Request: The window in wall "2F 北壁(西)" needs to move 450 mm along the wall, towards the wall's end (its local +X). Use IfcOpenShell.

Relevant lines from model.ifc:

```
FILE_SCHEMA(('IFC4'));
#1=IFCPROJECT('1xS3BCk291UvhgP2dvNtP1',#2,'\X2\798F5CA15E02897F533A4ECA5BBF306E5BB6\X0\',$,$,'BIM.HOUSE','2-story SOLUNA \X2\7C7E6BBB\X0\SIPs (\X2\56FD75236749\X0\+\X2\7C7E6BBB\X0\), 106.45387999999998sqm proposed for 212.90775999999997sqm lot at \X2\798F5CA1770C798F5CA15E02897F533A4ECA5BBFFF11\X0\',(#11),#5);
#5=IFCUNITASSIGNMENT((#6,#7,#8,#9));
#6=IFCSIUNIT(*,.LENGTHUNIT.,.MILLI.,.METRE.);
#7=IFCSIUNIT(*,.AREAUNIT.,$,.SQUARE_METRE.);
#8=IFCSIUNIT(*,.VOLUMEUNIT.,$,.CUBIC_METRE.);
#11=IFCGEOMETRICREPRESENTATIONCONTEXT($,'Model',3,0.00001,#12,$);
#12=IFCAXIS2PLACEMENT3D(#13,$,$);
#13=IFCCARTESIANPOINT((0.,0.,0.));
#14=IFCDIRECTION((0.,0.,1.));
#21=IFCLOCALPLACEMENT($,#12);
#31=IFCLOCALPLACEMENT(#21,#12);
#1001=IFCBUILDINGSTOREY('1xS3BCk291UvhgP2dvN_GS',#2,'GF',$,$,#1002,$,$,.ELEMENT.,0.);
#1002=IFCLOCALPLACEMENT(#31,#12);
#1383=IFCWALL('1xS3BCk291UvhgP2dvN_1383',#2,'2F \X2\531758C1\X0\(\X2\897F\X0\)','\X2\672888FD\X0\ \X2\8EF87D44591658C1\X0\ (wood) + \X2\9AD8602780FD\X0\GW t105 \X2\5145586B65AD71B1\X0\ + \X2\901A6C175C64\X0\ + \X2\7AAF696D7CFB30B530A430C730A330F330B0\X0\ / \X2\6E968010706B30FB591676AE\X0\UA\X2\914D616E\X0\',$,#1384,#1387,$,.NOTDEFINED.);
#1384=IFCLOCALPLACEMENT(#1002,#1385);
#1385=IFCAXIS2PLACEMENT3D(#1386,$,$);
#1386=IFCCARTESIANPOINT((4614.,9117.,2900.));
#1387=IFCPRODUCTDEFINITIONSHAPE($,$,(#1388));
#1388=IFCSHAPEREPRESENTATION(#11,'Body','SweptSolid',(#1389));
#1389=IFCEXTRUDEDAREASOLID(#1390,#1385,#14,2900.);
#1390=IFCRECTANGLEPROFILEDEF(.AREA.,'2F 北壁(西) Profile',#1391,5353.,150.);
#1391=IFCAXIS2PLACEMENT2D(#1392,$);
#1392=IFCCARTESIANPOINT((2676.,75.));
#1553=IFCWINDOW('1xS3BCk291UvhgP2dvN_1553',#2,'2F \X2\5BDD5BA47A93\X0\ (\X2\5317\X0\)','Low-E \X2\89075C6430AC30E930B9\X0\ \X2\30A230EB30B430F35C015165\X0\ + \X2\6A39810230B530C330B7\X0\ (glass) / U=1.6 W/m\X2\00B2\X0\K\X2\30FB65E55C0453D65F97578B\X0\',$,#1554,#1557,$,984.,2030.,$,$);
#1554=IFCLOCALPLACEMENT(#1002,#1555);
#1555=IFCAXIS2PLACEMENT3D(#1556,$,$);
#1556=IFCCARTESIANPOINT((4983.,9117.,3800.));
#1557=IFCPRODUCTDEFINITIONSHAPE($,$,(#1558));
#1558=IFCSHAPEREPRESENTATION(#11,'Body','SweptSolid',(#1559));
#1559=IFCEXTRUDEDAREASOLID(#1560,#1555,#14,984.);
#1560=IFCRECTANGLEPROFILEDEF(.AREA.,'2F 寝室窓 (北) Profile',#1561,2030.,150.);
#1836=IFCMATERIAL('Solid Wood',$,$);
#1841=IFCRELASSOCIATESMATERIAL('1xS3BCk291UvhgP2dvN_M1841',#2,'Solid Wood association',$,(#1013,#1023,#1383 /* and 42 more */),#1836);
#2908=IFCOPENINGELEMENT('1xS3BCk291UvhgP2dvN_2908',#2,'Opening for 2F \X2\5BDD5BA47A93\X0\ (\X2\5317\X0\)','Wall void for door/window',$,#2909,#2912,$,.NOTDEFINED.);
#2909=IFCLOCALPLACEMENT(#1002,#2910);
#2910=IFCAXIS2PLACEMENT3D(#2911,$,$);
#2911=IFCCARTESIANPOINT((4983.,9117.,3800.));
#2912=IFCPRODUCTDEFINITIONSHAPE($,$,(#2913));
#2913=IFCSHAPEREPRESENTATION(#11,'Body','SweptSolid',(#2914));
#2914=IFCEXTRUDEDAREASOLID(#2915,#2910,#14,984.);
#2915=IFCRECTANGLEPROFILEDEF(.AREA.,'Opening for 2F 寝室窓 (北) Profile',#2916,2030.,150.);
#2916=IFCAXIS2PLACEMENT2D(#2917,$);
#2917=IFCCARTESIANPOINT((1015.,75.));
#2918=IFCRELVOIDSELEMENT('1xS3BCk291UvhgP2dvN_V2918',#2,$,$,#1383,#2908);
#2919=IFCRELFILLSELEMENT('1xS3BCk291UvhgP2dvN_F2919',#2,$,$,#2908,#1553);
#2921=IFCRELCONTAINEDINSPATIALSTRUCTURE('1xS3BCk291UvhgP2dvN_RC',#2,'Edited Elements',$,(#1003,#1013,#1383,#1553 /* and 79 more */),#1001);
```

```python
import ifcopenshell
import ifcopenshell.api.geometry
import ifcopenshell.util.placement

model = ifcopenshell.open("model.ifc")

window = model.by_id(1553)
opening = window.FillsVoids[0].RelatingOpeningElement
wall = opening.VoidsElements[0].RelatingBuildingElement

wall_matrix = ifcopenshell.util.placement.get_local_placement(wall.ObjectPlacement)
shift = wall_matrix[:3, 0] * 450.0
before = ifcopenshell.util.placement.get_local_placement(window.ObjectPlacement)[:3, 3].copy()

# The window is not placed relative to its opening, so move both.
for product in (opening, window):
    matrix = ifcopenshell.util.placement.get_local_placement(product.ObjectPlacement)
    matrix[:3, 3] += shift
    ifcopenshell.api.geometry.edit_object_placement(model, product=product, matrix=matrix, is_si=False)

after = ifcopenshell.util.placement.get_local_placement(window.ObjectPlacement)[:3, 3]
print("window moved by", (after - before).round(3) + 0.0)

model.write("model_v2.ifc")
```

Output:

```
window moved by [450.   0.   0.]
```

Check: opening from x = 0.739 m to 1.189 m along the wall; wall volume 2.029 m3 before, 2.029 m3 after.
